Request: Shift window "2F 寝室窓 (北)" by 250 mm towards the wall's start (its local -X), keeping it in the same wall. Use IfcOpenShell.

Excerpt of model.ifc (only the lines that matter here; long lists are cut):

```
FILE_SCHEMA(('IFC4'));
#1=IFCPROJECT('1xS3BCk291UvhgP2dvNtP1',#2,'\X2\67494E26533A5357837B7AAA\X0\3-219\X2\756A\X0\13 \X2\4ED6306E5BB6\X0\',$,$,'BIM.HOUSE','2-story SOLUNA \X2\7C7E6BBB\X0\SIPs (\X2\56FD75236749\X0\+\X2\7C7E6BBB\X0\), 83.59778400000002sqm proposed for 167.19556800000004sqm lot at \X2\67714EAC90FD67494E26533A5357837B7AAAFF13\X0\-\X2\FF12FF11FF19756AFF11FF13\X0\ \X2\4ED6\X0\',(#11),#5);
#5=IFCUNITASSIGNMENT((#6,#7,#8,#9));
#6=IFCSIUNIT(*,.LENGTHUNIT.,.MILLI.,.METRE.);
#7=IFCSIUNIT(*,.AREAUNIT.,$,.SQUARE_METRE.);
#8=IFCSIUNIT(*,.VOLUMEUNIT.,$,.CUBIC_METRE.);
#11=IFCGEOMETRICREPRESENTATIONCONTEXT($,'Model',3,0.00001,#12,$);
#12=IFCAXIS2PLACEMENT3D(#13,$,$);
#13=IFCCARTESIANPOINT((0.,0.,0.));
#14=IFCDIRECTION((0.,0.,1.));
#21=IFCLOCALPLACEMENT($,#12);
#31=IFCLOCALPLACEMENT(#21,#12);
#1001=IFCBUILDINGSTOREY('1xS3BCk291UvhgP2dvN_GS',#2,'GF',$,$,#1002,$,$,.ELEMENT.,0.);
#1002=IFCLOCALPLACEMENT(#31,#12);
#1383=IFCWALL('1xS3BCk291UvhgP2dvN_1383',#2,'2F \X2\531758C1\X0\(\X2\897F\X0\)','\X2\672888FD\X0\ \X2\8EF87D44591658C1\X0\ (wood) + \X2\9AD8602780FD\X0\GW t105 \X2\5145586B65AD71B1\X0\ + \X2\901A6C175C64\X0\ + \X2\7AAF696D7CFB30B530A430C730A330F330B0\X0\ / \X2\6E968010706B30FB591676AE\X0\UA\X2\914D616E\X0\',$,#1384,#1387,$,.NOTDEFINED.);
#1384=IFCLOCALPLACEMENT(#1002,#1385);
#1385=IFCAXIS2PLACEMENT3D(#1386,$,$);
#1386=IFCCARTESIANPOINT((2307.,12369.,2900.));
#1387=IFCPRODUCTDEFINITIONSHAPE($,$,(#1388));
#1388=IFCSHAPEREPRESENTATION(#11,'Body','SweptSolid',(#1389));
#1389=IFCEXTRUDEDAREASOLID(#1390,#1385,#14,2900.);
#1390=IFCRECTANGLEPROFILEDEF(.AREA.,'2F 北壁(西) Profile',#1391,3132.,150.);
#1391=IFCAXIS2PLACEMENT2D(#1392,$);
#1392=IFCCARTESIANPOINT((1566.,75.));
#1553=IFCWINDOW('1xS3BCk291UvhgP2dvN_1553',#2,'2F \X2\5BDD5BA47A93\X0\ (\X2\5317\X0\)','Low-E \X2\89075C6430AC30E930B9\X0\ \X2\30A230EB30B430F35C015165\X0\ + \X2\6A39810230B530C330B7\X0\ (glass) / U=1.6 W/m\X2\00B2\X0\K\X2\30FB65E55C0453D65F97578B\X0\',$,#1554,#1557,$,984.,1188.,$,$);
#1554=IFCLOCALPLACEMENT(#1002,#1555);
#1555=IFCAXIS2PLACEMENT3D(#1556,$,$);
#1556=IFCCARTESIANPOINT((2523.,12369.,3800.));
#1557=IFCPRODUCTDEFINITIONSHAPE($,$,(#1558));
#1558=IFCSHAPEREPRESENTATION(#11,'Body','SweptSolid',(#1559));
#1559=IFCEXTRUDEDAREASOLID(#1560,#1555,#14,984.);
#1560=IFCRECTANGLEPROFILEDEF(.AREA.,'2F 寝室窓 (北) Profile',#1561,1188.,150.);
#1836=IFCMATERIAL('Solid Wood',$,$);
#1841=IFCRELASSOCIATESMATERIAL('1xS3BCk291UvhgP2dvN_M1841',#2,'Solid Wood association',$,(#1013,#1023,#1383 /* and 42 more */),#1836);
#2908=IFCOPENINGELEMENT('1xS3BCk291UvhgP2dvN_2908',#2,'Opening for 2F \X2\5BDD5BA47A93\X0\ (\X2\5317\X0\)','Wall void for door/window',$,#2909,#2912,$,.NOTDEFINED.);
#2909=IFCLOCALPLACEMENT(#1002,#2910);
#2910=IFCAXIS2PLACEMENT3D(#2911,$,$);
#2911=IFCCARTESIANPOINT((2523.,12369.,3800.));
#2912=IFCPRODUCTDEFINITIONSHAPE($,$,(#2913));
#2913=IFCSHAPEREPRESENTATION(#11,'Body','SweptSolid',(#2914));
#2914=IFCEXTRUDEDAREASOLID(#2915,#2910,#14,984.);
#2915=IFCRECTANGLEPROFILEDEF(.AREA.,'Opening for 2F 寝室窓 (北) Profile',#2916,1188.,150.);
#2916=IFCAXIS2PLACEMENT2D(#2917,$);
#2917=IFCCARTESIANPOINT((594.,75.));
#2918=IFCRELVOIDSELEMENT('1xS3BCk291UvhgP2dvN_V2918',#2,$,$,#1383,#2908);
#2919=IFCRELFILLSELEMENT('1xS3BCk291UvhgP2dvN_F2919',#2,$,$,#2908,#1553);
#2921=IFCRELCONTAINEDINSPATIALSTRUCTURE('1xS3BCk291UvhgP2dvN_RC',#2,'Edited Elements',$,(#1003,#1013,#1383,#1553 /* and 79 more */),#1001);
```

```python
import ifcopenshell
import ifcopenshell.api.geometry
import ifcopenshell.util.placement
import ifcopenshell.util.unit

model = ifcopenshell.open("model.ifc")
unit_scale = ifcopenshell.util.unit.calculate_unit_scale(model)

window = model.by_id(1553)
opening = window.FillsVoids[0].RelatingOpeningElement
wall = opening.VoidsElements[0].RelatingBuildingElement

wall_matrix = ifcopenshell.util.placement.get_local_placement(wall.ObjectPlacement)
shift = wall_matrix[:3, 0] * -0.25 / unit_scale
before = ifcopenshell.util.placement.get_local_placement(window.ObjectPlacement)[:3, 3].copy()

# The window is not placed relative to its opening, so move both.
for product in (opening, window):
    matrix = ifcopenshell.util.placement.get_local_placement(product.ObjectPlacement)
    matrix[:3, 3] += shift
    ifcopenshell.api.geometry.edit_object_placement(model, product=product, matrix=matrix, is_si=False)

after = ifcopenshell.util.placement.get_local_placement(window.ObjectPlacement)[:3, 3]
print("window moved by", (after - before).round(3) + 0.0)

model.write("model_updated.ifc")
```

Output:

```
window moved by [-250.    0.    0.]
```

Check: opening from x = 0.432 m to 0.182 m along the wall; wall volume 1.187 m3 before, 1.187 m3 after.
